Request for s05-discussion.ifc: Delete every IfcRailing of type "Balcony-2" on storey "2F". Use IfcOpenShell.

First a look at what the model holds.

```python
import ifcopenshell
import ifcopenshell.util.element

model = ifcopenshell.open("s05-discussion.ifc")
print(model.schema)
storey = next(s for s in model.by_type("IfcBuildingStorey") if s.Name == "2F")
railings = [e for e in ifcopenshell.util.element.get_decomposition(storey) if e.is_a("IfcRailing")]
seen = {}
for e in railings:
    element_type = ifcopenshell.util.element.get_type(e)
    name = element_type.Name if element_type not in (None, e) else None
    seen[name] = seen.get(name, 0) + 1
for name, count in sorted(seen.items(), key=str):
    print(count, "x", name)
```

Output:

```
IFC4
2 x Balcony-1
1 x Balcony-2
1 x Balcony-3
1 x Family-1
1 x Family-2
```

```python
import ifcopenshell
import ifcopenshell.api.root
import ifcopenshell.util.element

model = ifcopenshell.open("s05-discussion.ifc")

storey = next(s for s in model.by_type("IfcBuildingStorey") if s.Name == "2F")
railings = [e for e in ifcopenshell.util.element.get_decomposition(storey) if e.is_a("IfcRailing")]
targets = [e for e in railings if (t := ifcopenshell.util.element.get_type(e)) not in (None, e) and t.Name == "Balcony-2"]

for e in targets:
    ifcopenshell.api.root.remove_product(model, product=e)
print(len(targets), "removed")

model.write("s05-discussion_updated.ifc")
```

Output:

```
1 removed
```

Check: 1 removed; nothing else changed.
